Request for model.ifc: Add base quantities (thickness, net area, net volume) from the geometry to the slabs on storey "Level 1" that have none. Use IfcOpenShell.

First a look at what the model holds.

```python
import ifcopenshell
import ifcopenshell.util.element
import ifcopenshell.util.unit

model = ifcopenshell.open("model.ifc")
print(model.schema)
for unit_type in ("LENGTHUNIT", "AREAUNIT", "VOLUMEUNIT"):
    print(unit_type, ifcopenshell.util.unit.calculate_unit_scale(model, unit_type))
storey = next(s for s in model.by_type("IfcBuildingStorey") if s.Name == "Level 1")
slabs = [e for e in ifcopenshell.util.element.get_decomposition(storey) if e.is_a("IfcSlab")]
for e in sorted(slabs, key=lambda e: e.id()):
    print(e.id(), e.is_a(), e.Name, list(ifcopenshell.util.element.get_psets(e, qtos_only=True)), sep=" | ")
```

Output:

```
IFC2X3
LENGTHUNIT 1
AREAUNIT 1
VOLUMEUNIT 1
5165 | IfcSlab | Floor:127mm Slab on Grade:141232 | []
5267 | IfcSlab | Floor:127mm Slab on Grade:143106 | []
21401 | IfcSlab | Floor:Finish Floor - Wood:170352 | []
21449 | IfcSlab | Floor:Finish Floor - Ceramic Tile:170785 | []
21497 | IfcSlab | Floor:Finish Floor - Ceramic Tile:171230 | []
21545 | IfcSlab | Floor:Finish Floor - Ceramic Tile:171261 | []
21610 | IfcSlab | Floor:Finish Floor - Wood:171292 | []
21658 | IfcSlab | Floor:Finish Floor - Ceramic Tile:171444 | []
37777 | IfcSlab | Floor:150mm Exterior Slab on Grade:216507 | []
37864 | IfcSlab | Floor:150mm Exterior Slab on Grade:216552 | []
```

```python
import ifcopenshell
import ifcopenshell.api.pset
import ifcopenshell.geom
import ifcopenshell.util.element
import ifcopenshell.util.shape
import ifcopenshell.util.unit

model = ifcopenshell.open("model.ifc")
unit_scale = ifcopenshell.util.unit.calculate_unit_scale(model)
area_scale = ifcopenshell.util.unit.calculate_unit_scale(model, "AREAUNIT")
volume_scale = ifcopenshell.util.unit.calculate_unit_scale(model, "VOLUMEUNIT")
settings = ifcopenshell.geom.settings()

storey = next(s for s in model.by_type("IfcBuildingStorey") if s.Name == "Level 1")
slabs = [e for e in ifcopenshell.util.element.get_decomposition(storey) if e.is_a("IfcSlab")]

for e in sorted(slabs, key=lambda e: e.id()):
    if ifcopenshell.util.element.get_psets(e, qtos_only=True, should_inherit=False):
        continue
    # Geometry comes back in metres, in the element's own axes.
    shape = ifcopenshell.geom.create_shape(settings, e)
    values = {
        "Width": ifcopenshell.util.shape.get_z(shape.geometry) / unit_scale,
        "NetArea": ifcopenshell.util.shape.get_footprint_area(shape.geometry) / area_scale,
        "NetVolume": ifcopenshell.util.shape.get_volume(shape.geometry) / volume_scale,
    }
    qto = ifcopenshell.api.pset.add_qto(model, product=e, name="BaseQuantities")
    ifcopenshell.api.pset.edit_qto(model, qto=qto, properties=values)
    print(e.id(), {k: round(v, 3) for k, v in values.items()})

model.write("model_edited.ifc")
```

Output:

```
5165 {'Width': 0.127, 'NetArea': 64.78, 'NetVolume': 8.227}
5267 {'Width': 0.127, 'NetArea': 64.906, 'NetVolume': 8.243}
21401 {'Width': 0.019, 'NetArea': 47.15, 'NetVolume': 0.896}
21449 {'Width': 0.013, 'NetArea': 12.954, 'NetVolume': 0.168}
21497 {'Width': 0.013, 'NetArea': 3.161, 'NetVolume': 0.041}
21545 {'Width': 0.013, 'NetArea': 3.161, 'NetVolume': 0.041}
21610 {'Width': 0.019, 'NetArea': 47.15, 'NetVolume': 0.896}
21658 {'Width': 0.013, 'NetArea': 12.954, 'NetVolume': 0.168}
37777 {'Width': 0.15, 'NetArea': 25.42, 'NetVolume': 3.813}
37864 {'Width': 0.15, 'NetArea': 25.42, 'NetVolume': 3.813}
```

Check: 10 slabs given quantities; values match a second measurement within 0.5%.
